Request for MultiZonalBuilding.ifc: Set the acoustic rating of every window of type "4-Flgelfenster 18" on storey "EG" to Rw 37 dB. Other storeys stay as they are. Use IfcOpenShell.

First a look at what the model holds.

```python
import ifcopenshell
import ifcopenshell.util.element

model = ifcopenshell.open("MultiZonalBuilding.ifc")
print(model.schema)
storey = next(s for s in model.by_type("IfcBuildingStorey") if s.Name == "EG")
windows = [e for e in ifcopenshell.util.element.get_decomposition(storey) if e.is_a("IfcWindow")]
seen = {}
for e in windows:
    element_type = ifcopenshell.util.element.get_type(e)
    key = (element_type.Name if element_type != e and element_type else None, ifcopenshell.util.element.get_pset(e, "Pset_WindowCommon", "AcousticRating"))
    seen[key] = seen.get(key, 0) + 1
for (name, value), count in sorted(seen.items(), key=str):
    print(count, "x", name, "|", value)
```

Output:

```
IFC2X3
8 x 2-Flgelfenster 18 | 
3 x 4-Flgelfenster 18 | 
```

```python
import ifcopenshell
import ifcopenshell.api.pset
import ifcopenshell.util.element

model = ifcopenshell.open("MultiZonalBuilding.ifc")

storey = next(s for s in model.by_type("IfcBuildingStorey") if s.Name == "EG")
windows = [e for e in ifcopenshell.util.element.get_decomposition(storey) if e.is_a("IfcWindow")]

count = 0
for e in windows:
    element_type = ifcopenshell.util.element.get_type(e)
    if element_type in (None, e) or element_type.Name != '4-Fl\x9fgelfenster 18':
        continue
    # add_pset returns the element's existing set when there is one.
    pset = ifcopenshell.api.pset.add_pset(model, product=e, name="Pset_WindowCommon")
    ifcopenshell.api.pset.edit_pset(model, pset=pset, properties={"AcousticRating": "Rw 37 dB"})
    count += 1

print(count, "windows updated")

model.write("MultiZonalBuilding_edited.ifc")
```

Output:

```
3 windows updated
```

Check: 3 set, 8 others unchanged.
